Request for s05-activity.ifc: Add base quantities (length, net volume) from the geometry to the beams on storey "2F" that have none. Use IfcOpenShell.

First a look at what the model holds.

```python
import ifcopenshell
import ifcopenshell.util.element
import ifcopenshell.util.unit

model = ifcopenshell.open("s05-activity.ifc")
print(model.schema)
for unit_type in ("LENGTHUNIT", "AREAUNIT", "VOLUMEUNIT"):
    print(unit_type, ifcopenshell.util.unit.calculate_unit_scale(model, unit_type))
storey = next(s for s in model.by_type("IfcBuildingStorey") if s.Name == "2F")
beams = [e for e in ifcopenshell.util.element.get_decomposition(storey) if e.is_a("IfcBeam")]
for e in sorted(beams, key=lambda e: e.id()):
    print(e.id(), e.is_a(), e.Name, list(ifcopenshell.util.element.get_psets(e, qtos_only=True)), sep=" | ")
```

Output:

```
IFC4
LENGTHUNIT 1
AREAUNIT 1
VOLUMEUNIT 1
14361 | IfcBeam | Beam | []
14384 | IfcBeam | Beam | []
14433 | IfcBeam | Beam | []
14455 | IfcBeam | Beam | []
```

```python
import ifcopenshell
import ifcopenshell.api.pset
import ifcopenshell.geom
import ifcopenshell.util.element
import ifcopenshell.util.shape
import ifcopenshell.util.unit

model = ifcopenshell.open("s05-activity.ifc")
unit_scale = ifcopenshell.util.unit.calculate_unit_scale(model)
volume_scale = ifcopenshell.util.unit.calculate_unit_scale(model, "VOLUMEUNIT")
settings = ifcopenshell.geom.settings()

storey = next(s for s in model.by_type("IfcBuildingStorey") if s.Name == "2F")
beams = [e for e in ifcopenshell.util.element.get_decomposition(storey) if e.is_a("IfcBeam")]

for e in sorted(beams, key=lambda e: e.id()):
    if ifcopenshell.util.element.get_psets(e, qtos_only=True, should_inherit=False):
        continue
    # Geometry comes back in metres, in the element's own axes.
    shape = ifcopenshell.geom.create_shape(settings, e)
    values = {
        "Length": ifcopenshell.util.shape.get_max_xyz(shape.geometry) / unit_scale,
        "NetVolume": ifcopenshell.util.shape.get_volume(shape.geometry) / volume_scale,
    }
    qto = ifcopenshell.api.pset.add_qto(model, product=e, name="Qto_BeamBaseQuantities")
    ifcopenshell.api.pset.edit_qto(model, qto=qto, properties=values)
    print(e.id(), {k: round(v, 3) for k, v in values.items()})

model.write("s05-activity_v2.ifc")
```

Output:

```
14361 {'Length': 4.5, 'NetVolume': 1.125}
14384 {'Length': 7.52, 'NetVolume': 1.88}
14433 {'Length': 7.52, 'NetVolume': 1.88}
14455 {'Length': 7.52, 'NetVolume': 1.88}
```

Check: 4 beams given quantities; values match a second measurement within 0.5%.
